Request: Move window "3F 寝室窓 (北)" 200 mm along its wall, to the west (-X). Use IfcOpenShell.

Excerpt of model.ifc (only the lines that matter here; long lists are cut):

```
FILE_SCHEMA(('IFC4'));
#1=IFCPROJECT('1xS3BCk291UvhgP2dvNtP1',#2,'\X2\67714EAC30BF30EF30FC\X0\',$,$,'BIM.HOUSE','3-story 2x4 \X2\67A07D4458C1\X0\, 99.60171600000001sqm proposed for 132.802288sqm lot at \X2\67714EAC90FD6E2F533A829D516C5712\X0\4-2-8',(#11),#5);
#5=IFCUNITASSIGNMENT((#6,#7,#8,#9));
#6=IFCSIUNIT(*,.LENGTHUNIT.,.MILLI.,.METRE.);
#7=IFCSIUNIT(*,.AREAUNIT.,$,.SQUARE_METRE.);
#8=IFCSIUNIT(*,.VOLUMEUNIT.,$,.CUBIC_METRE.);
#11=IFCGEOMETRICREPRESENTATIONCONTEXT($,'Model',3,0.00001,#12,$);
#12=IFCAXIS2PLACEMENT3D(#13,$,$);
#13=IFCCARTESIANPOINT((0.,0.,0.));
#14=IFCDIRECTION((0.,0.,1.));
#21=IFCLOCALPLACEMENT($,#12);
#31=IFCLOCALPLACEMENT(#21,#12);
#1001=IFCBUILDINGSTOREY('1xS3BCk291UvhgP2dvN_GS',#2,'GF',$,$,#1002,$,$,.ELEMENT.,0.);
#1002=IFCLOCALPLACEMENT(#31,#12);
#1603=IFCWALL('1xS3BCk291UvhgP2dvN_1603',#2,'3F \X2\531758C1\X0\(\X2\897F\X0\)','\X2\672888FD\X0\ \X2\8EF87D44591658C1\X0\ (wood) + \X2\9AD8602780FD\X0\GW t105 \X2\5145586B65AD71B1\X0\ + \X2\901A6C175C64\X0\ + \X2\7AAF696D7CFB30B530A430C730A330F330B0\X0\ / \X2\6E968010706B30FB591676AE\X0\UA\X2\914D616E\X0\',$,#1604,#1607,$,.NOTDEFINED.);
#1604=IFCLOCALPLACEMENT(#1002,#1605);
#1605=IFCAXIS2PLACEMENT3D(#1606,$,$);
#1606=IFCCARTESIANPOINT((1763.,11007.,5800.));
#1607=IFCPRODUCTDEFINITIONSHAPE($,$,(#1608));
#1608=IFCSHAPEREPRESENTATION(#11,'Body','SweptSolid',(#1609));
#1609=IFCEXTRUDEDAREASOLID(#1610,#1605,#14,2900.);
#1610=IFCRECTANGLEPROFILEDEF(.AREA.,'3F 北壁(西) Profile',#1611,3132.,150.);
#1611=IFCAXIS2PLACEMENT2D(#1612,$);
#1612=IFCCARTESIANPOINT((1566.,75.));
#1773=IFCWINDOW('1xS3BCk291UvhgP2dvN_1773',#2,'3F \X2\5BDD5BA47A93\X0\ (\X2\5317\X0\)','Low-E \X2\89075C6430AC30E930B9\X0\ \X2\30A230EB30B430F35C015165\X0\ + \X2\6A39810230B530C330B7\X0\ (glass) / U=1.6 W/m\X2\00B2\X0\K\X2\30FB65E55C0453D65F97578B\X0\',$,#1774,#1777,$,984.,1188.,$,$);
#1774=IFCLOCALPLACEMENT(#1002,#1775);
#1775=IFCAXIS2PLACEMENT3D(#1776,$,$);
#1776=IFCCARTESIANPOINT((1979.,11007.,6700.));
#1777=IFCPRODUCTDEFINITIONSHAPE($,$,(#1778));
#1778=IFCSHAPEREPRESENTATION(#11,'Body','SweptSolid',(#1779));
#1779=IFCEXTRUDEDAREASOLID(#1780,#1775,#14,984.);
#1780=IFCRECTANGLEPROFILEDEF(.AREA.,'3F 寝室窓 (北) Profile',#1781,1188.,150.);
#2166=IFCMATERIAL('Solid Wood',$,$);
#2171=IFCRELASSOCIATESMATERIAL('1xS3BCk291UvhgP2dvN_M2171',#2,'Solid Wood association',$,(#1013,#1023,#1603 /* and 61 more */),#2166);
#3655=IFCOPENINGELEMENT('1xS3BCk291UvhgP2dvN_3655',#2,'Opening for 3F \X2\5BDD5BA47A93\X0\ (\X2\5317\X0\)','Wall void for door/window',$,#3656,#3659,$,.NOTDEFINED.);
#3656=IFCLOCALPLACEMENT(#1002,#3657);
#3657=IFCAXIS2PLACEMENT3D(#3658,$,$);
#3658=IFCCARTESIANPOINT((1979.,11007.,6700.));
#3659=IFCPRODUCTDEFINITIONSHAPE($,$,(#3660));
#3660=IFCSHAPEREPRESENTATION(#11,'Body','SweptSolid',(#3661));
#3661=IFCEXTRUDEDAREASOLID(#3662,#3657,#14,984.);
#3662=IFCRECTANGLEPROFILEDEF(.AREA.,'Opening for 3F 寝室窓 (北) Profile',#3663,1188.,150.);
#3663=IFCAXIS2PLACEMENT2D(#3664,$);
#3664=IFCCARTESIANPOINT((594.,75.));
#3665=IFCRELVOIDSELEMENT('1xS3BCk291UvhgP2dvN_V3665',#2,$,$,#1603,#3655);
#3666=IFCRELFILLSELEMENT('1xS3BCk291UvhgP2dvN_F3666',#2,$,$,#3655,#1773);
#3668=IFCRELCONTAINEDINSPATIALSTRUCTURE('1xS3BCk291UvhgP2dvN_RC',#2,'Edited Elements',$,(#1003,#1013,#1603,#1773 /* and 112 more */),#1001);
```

```python
import ifcopenshell
import ifcopenshell.api.geometry
import ifcopenshell.util.placement
import ifcopenshell.util.unit

model = ifcopenshell.open("model.ifc")
unit_scale = ifcopenshell.util.unit.calculate_unit_scale(model)

window = model.by_id(1773)
opening = window.FillsVoids[0].RelatingOpeningElement
wall = opening.VoidsElements[0].RelatingBuildingElement

wall_matrix = ifcopenshell.util.placement.get_local_placement(wall.ObjectPlacement)
shift = wall_matrix[:3, 0] * -0.2 / unit_scale
before = ifcopenshell.util.placement.get_local_placement(window.ObjectPlacement)[:3, 3].copy()

# The window is not placed relative to its opening, so move both.
for product in (opening, window):
    matrix = ifcopenshell.util.placement.get_local_placement(product.ObjectPlacement)
    matrix[:3, 3] += shift
    ifcopenshell.api.geometry.edit_object_placement(model, product=product, matrix=matrix, is_si=False)

after = ifcopenshell.util.placement.get_local_placement(window.ObjectPlacement)[:3, 3]
print("window moved by", (after - before).round(3) + 0.0)

model.write("model_rev.ifc")
```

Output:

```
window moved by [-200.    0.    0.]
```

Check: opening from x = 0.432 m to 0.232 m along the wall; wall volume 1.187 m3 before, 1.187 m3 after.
